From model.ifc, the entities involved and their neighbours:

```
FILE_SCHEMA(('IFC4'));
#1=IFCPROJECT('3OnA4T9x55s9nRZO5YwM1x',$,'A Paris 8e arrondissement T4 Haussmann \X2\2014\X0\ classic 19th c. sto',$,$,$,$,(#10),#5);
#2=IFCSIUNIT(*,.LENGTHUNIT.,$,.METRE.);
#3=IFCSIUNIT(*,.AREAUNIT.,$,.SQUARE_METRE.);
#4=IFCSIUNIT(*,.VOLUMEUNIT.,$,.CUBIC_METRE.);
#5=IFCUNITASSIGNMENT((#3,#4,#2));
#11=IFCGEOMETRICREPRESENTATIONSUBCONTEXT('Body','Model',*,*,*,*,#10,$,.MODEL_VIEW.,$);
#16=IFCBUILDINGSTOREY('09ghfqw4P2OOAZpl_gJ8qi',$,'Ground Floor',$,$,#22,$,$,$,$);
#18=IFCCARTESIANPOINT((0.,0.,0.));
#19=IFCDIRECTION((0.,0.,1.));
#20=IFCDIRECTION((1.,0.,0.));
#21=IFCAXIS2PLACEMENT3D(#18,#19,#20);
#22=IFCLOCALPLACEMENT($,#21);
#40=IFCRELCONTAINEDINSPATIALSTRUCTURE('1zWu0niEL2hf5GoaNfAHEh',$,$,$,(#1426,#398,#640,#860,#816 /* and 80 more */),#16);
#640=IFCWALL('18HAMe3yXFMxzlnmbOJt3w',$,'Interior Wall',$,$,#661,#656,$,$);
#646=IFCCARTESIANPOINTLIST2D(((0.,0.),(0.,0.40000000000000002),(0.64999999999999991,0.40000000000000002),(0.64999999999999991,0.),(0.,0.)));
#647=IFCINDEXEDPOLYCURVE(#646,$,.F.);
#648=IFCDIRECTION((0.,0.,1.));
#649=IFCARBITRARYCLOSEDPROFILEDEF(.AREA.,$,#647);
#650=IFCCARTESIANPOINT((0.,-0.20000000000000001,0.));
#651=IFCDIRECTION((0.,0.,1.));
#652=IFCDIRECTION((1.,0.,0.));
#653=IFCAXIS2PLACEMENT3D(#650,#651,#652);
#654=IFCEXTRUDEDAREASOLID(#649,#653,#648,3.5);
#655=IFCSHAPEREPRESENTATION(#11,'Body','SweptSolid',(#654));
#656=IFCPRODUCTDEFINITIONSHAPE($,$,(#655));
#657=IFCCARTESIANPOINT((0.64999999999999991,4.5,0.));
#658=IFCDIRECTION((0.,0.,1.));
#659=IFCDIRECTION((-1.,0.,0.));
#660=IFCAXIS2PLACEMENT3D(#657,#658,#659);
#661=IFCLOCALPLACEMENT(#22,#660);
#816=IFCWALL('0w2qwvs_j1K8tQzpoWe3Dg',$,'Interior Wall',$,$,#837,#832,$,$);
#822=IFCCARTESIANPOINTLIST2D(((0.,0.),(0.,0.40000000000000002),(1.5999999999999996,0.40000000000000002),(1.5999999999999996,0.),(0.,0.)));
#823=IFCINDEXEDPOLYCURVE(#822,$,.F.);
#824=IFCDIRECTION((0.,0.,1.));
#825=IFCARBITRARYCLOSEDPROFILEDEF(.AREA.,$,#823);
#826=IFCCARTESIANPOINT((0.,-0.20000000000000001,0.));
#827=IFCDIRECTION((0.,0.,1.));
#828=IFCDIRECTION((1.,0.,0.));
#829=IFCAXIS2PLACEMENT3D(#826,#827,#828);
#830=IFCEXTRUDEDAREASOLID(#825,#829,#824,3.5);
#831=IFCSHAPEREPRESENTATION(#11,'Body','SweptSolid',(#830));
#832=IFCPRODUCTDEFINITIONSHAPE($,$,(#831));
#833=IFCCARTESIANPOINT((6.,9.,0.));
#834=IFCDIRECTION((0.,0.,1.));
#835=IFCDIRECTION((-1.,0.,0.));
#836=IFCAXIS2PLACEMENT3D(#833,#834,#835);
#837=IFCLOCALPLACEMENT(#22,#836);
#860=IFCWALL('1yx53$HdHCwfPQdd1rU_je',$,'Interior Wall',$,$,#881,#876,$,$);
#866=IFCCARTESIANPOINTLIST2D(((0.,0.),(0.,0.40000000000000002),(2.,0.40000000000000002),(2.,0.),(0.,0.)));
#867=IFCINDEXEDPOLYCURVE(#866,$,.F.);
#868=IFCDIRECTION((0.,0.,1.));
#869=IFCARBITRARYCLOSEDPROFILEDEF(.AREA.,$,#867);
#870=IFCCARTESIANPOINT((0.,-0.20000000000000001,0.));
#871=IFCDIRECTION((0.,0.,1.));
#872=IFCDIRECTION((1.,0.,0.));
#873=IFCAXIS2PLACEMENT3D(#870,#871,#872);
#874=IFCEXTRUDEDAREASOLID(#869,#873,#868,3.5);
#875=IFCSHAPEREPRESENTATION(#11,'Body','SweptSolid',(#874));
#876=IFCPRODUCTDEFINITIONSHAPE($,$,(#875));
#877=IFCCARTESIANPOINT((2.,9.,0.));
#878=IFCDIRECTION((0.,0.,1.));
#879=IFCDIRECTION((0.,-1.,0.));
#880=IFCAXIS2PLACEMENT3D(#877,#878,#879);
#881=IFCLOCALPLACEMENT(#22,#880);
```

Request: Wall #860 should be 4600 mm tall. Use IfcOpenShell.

```python
import ifcopenshell
import ifcopenshell.geom
import ifcopenshell.util.representation
import ifcopenshell.util.shape

model = ifcopenshell.open("model.ifc")
settings = ifcopenshell.geom.settings()


def volume(element):
    """Net volume in cubic metres, openings subtracted."""
    shape = ifcopenshell.geom.create_shape(settings, element)
    return ifcopenshell.util.shape.get_volume(shape.geometry)


wall = model.by_guid("1yx53$HdHCwfPQdd1rU_je")
before = volume(wall)

body = ifcopenshell.util.representation.get_representation(wall, "Model", "Body")
solid = body.Items[0]
old_height = solid.Depth
solid.Depth = 4.6
after = volume(wall)

print(f"height {old_height:g} -> {solid.Depth:g}, volume {before:.3f} -> {after:.3f} m3")

model.write("model_updated.ifc")
```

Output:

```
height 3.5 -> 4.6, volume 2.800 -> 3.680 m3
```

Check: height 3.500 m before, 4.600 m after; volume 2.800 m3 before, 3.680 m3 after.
